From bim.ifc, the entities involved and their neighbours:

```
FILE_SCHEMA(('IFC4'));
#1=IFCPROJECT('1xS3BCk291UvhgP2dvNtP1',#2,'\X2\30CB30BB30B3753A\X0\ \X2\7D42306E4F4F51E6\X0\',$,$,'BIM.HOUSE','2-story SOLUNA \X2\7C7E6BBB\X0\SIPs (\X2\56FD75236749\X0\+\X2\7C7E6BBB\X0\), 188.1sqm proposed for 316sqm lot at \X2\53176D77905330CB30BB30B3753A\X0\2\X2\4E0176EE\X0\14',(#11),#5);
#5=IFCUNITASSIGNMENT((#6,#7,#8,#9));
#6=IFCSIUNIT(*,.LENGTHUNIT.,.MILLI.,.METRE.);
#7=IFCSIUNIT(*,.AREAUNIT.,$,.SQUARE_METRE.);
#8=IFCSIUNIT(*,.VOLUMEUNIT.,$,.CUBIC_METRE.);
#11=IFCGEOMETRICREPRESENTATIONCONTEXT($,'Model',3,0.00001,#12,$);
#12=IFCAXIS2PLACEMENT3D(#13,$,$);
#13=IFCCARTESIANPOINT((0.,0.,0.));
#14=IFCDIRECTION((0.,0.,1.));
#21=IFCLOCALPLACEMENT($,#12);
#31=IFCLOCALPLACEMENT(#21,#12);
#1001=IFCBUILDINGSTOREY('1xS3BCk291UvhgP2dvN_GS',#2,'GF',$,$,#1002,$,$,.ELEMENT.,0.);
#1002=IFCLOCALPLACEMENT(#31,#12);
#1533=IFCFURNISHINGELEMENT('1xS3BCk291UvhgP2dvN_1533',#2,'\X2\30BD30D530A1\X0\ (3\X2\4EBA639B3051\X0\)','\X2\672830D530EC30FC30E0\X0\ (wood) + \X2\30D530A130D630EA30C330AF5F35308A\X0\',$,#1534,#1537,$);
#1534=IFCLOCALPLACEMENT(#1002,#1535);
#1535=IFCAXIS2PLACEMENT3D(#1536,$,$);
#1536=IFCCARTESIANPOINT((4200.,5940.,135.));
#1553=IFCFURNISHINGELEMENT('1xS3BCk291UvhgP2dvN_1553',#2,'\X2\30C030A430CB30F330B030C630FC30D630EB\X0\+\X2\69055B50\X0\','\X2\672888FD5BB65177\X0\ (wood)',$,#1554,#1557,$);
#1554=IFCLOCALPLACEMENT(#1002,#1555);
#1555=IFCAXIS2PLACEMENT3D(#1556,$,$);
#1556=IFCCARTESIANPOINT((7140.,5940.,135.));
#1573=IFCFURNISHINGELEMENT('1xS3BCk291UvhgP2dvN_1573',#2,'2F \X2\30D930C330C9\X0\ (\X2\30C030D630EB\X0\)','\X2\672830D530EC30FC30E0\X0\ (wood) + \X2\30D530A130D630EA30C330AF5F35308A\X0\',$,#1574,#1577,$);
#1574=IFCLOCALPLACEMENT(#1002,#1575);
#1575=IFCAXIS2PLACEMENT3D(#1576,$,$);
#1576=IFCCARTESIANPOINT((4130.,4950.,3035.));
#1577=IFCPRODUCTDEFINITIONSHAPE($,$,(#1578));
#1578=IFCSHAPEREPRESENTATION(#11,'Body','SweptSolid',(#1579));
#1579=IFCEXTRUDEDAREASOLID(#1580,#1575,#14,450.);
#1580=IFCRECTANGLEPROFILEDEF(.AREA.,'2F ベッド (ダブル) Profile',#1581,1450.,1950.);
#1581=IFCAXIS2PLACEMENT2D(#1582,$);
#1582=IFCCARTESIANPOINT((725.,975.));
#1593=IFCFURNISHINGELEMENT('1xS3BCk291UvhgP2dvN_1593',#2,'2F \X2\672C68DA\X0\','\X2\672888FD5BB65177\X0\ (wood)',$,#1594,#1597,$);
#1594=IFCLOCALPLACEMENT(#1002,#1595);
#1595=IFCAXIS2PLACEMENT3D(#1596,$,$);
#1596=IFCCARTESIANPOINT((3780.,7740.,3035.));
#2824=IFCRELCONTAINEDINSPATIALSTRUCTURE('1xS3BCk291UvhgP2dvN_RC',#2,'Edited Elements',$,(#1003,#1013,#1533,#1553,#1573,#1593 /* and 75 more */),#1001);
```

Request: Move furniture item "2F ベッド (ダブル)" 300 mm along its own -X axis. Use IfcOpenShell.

```python
import ifcopenshell
import ifcopenshell.api.geometry
import ifcopenshell.util.placement
import ifcopenshell.util.unit

model = ifcopenshell.open("bim.ifc")
unit_scale = ifcopenshell.util.unit.calculate_unit_scale(model)

item = model.by_guid("1xS3BCk291UvhgP2dvN_1573")
matrix = ifcopenshell.util.placement.get_local_placement(item.ObjectPlacement)
matrix[:3, 3] -= matrix[:3, 0] * 0.3 / unit_scale
ifcopenshell.api.geometry.edit_object_placement(model, product=item, matrix=matrix, is_si=False)

print(ifcopenshell.util.placement.get_local_placement(item.ObjectPlacement).round(3) + 0.0)

model.write("bim_v2.ifc")
```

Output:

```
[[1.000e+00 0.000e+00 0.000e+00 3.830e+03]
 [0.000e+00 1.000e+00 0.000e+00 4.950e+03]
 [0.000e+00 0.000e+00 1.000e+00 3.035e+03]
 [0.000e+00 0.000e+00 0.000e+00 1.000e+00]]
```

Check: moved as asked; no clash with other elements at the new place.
